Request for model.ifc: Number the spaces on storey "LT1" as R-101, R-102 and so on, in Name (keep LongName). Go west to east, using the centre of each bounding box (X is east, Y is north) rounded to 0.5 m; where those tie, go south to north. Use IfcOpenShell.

First a look at what the model holds.

```python
import ifcopenshell
import ifcopenshell.util.element
import ifcopenshell.util.placement

model = ifcopenshell.open("model.ifc")
print(model.schema)
storey = next(s for s in model.by_type("IfcBuildingStorey") if s.Name == "LT1")
spaces = [e for e in ifcopenshell.util.element.get_decomposition(storey) if e.is_a("IfcSpace")]
for e in sorted(spaces, key=lambda e: e.id()):
    origin = ifcopenshell.util.placement.get_local_placement(e.ObjectPlacement)[:3, 3]
    print(e.id(), e.Name, e.LongName, origin.round(2) + 0.0, sep=" | ")
```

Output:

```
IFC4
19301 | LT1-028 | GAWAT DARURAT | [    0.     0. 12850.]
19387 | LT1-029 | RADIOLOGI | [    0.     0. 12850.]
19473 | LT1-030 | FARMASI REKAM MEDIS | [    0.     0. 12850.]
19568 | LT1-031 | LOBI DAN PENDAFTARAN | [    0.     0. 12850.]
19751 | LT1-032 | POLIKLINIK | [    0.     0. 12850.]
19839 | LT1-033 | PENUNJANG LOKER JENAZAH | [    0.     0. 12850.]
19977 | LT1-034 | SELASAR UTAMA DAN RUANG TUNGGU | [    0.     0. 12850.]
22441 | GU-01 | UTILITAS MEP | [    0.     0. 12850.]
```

```python
import ifcopenshell
import ifcopenshell.geom
import ifcopenshell.util.element
import ifcopenshell.util.shape

model = ifcopenshell.open("model.ifc")
settings = ifcopenshell.geom.settings()
settings.set("use-world-coords", True)


def centre(element):
    shape = ifcopenshell.geom.create_shape(settings, element)
    return ifcopenshell.util.shape.get_bbox_centroid(shape.geometry)


storey = next(s for s in model.by_type("IfcBuildingStorey") if s.Name == "LT1")
spaces = [e for e in ifcopenshell.util.element.get_decomposition(storey) if e.is_a("IfcSpace")]

# Insertion points can sit at a corner or the storey origin, so sort by the geometry (in metres).
centres = {e: centre(e) for e in spaces}
spaces.sort(key=lambda e: (round(centres[e][0] / 0.5), centres[e][1]))

for i, e in enumerate(spaces, start=1):
    number = f"R-1{i:02d}"
    e.Name = number
    print(e.id(), number)

model.write("model_rev.ifc")
```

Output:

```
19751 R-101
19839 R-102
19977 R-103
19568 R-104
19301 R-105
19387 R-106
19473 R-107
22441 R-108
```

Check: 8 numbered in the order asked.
